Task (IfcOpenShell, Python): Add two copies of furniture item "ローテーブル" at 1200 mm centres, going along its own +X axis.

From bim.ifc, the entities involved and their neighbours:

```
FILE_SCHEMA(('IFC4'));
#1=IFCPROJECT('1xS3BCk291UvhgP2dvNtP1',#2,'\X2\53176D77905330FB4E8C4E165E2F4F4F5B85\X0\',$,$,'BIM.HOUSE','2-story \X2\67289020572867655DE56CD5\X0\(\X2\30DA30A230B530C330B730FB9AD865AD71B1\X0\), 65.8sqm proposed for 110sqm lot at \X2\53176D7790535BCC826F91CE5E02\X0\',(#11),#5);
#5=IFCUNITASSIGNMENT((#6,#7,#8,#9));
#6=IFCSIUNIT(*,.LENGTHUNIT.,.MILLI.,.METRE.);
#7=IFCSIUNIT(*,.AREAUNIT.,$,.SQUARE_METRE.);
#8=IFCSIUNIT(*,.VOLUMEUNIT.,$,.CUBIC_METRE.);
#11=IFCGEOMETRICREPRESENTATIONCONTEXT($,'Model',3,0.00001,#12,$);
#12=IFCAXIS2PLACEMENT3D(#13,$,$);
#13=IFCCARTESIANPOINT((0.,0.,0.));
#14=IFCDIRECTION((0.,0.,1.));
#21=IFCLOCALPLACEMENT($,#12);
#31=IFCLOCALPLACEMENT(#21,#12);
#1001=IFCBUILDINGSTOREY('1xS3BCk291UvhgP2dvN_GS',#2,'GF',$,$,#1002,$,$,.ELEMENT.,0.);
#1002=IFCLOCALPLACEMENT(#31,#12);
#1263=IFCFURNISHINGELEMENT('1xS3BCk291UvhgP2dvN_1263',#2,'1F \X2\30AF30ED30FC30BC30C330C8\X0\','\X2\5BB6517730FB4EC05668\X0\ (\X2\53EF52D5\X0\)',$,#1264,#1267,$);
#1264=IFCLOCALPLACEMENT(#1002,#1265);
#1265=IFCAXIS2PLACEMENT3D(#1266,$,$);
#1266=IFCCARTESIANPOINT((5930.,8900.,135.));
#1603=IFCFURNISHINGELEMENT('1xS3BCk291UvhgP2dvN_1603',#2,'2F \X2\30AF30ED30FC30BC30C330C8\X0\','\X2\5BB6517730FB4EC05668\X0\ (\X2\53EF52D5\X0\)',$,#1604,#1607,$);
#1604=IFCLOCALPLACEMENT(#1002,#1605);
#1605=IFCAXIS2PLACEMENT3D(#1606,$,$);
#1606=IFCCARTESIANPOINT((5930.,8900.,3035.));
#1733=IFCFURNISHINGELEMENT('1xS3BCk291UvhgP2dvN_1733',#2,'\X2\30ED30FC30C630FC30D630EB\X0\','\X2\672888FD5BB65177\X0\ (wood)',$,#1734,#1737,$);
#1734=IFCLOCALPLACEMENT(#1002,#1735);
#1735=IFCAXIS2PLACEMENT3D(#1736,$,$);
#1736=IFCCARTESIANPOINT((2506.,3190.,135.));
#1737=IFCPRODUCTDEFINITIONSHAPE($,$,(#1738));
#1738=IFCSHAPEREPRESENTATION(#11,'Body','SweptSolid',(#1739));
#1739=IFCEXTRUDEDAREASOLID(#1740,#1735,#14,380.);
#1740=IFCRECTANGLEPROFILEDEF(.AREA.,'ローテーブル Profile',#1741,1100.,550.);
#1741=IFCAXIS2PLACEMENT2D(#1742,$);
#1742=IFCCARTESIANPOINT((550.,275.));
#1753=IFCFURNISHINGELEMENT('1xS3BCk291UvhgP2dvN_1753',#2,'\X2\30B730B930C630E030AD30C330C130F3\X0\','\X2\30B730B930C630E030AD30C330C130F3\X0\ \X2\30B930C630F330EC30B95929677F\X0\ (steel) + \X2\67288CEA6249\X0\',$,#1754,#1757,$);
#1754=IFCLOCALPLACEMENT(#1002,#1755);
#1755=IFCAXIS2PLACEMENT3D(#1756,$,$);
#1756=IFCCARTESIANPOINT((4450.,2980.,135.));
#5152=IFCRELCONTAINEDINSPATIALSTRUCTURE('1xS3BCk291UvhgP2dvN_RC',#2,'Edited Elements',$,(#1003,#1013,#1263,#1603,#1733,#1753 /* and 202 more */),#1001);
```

```python
import ifcopenshell
import ifcopenshell.api.geometry
import ifcopenshell.api.root
import ifcopenshell.util.element
import ifcopenshell.util.placement
import ifcopenshell.util.unit

model = ifcopenshell.open("bim.ifc")
unit_scale = ifcopenshell.util.unit.calculate_unit_scale(model)


def reuse_history(source, copy):
    """copy_class also copies each property set's owner history, people and application; keep the originals."""
    for rel in copy.IsDefinedBy:
        if rel.is_a("IfcRelDefinesByProperties") and (history := rel.RelatingPropertyDefinition.OwnerHistory):
            rel.RelatingPropertyDefinition.OwnerHistory = source.OwnerHistory
            ifcopenshell.util.element.remove_deep2(model, history)


source = model.by_guid("1xS3BCk291UvhgP2dvN_1733")
base = ifcopenshell.util.placement.get_local_placement(source.ObjectPlacement)
step = base[:3, 0] * 1.2 / unit_scale

for i in range(1, 3):
    copy = ifcopenshell.api.root.copy_class(model, product=source)
    copy.Representation = ifcopenshell.util.element.copy_deep(
        model, source.Representation, exclude=["IfcGeometricRepresentationContext", "IfcRepresentationMap"]
    )
    reuse_history(source, copy)
    matrix = base.copy()
    matrix[:3, 3] += i * step
    print("added at", matrix[:3, 3].round(3) + 0.0)
    ifcopenshell.api.geometry.edit_object_placement(model, product=copy, matrix=matrix, is_si=False)

model.write("bim_updated.ifc")
```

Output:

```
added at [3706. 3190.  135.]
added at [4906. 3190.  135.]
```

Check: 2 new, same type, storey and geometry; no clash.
